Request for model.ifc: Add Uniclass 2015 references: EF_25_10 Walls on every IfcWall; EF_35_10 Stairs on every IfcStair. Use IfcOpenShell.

First a look at what the model holds.

```python
import ifcopenshell

model = ifcopenshell.open("model.ifc")
print(model.schema)
print("classifications:", [c.Name for c in model.by_type("IfcClassification")])
for ifc_class in ("IfcDoor", "IfcRoof", "IfcStair", "IfcWall", "IfcWindow"):
    print(ifc_class, len(model.by_type(ifc_class)))
```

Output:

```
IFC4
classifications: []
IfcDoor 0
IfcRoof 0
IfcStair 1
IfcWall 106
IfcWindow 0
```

```python
import ifcopenshell
import ifcopenshell.api.classification

model = ifcopenshell.open("model.ifc")

system = ifcopenshell.api.classification.add_classification(model, classification="Uniclass 2015")

codes = {
    "IfcWall": ("EF_25_10", "Walls"),
    "IfcStair": ("EF_35_10", "Stairs"),
}
for ifc_class, (code, name) in codes.items():
    products = model.by_type(ifc_class)
    ifcopenshell.api.classification.add_reference(
        model, products=products, classification=system, identification=code, name=name
    )
    print(code, len(products))

model.write("model_updated.ifc")
```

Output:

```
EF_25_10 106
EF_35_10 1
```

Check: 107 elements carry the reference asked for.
